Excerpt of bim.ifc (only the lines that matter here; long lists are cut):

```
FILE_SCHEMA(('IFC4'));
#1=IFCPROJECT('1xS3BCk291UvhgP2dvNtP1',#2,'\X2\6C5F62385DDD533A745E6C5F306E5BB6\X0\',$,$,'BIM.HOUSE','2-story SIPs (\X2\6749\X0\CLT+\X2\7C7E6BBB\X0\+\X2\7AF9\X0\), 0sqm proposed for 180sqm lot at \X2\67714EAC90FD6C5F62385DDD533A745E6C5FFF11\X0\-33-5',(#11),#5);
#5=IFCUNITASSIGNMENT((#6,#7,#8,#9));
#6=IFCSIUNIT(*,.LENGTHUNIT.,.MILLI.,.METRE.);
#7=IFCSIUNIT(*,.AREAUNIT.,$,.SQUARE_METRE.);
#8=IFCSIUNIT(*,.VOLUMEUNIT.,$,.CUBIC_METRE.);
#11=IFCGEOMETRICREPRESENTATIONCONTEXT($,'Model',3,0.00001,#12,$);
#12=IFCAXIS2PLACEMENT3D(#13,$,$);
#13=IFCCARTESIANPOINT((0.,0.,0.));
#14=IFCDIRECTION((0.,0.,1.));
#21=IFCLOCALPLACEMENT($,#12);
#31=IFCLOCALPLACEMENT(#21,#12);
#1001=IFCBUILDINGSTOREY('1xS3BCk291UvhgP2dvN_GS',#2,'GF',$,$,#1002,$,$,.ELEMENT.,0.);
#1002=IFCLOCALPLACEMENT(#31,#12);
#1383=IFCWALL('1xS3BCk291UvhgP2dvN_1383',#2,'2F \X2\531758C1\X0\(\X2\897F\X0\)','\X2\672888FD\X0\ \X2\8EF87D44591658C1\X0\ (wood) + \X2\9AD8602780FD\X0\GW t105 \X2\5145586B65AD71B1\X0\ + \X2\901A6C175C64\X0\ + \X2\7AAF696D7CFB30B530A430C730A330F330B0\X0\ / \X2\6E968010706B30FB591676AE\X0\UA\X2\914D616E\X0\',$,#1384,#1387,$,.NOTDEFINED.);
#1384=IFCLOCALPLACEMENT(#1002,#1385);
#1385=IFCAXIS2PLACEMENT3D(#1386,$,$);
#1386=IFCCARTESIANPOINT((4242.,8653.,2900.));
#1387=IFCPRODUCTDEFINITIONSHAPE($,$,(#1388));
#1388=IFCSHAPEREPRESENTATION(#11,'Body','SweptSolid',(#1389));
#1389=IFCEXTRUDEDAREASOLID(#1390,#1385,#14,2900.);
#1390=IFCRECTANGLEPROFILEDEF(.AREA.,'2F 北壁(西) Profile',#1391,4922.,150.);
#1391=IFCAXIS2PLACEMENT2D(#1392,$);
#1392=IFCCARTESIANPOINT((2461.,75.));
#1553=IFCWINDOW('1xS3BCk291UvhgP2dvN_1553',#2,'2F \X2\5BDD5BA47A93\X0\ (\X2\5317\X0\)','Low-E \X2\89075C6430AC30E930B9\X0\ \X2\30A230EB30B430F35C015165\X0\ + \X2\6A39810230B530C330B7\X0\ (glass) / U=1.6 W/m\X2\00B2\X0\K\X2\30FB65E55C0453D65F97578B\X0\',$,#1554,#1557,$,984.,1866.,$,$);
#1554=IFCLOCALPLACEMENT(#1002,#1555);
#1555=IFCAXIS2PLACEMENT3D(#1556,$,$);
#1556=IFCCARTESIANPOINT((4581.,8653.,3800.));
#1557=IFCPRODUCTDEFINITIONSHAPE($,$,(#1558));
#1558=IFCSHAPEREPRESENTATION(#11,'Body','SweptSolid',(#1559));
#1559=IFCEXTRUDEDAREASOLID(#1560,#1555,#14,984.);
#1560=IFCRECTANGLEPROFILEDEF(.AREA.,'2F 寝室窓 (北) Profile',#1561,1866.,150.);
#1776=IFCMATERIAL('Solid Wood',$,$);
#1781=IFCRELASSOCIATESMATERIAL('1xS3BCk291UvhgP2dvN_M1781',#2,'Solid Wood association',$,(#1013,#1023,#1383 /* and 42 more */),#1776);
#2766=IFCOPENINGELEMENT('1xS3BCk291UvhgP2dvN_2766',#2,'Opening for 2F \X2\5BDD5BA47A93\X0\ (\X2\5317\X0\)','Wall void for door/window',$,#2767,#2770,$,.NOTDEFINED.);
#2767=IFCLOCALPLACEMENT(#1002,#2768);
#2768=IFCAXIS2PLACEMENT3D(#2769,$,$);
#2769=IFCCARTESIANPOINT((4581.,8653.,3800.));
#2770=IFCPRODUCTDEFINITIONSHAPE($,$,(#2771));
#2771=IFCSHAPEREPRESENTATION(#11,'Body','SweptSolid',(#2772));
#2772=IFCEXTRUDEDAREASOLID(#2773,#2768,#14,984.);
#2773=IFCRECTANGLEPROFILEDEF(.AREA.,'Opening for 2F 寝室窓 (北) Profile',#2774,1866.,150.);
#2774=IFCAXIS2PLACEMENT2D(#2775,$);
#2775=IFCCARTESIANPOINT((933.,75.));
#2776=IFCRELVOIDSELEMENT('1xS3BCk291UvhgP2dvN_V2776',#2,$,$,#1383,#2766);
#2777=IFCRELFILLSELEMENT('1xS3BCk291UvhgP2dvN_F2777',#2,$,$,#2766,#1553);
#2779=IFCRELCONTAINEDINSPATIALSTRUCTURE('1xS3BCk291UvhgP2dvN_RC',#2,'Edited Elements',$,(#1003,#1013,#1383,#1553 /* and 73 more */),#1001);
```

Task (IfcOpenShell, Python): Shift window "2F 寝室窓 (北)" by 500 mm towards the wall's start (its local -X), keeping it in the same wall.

```python
import ifcopenshell
import ifcopenshell.api.geometry
import ifcopenshell.util.placement
import ifcopenshell.util.unit

model = ifcopenshell.open("bim.ifc")
unit_scale = ifcopenshell.util.unit.calculate_unit_scale(model)

window = model.by_guid("1xS3BCk291UvhgP2dvN_1553")
opening = window.FillsVoids[0].RelatingOpeningElement
wall = opening.VoidsElements[0].RelatingBuildingElement

wall_matrix = ifcopenshell.util.placement.get_local_placement(wall.ObjectPlacement)
shift = wall_matrix[:3, 0] * -0.5 / unit_scale
before = ifcopenshell.util.placement.get_local_placement(window.ObjectPlacement)[:3, 3].copy()

# The window is not placed relative to its opening, so move both.
for product in (opening, window):
    matrix = ifcopenshell.util.placement.get_local_placement(product.ObjectPlacement)
    matrix[:3, 3] += shift
    ifcopenshell.api.geometry.edit_object_placement(model, product=product, matrix=matrix, is_si=False)

after = ifcopenshell.util.placement.get_local_placement(window.ObjectPlacement)[:3, 3]
print("window moved by", (after - before).round(3) + 0.0)

model.write("bim_updated.ifc")
```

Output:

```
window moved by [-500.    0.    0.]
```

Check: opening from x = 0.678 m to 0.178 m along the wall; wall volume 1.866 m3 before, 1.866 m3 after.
